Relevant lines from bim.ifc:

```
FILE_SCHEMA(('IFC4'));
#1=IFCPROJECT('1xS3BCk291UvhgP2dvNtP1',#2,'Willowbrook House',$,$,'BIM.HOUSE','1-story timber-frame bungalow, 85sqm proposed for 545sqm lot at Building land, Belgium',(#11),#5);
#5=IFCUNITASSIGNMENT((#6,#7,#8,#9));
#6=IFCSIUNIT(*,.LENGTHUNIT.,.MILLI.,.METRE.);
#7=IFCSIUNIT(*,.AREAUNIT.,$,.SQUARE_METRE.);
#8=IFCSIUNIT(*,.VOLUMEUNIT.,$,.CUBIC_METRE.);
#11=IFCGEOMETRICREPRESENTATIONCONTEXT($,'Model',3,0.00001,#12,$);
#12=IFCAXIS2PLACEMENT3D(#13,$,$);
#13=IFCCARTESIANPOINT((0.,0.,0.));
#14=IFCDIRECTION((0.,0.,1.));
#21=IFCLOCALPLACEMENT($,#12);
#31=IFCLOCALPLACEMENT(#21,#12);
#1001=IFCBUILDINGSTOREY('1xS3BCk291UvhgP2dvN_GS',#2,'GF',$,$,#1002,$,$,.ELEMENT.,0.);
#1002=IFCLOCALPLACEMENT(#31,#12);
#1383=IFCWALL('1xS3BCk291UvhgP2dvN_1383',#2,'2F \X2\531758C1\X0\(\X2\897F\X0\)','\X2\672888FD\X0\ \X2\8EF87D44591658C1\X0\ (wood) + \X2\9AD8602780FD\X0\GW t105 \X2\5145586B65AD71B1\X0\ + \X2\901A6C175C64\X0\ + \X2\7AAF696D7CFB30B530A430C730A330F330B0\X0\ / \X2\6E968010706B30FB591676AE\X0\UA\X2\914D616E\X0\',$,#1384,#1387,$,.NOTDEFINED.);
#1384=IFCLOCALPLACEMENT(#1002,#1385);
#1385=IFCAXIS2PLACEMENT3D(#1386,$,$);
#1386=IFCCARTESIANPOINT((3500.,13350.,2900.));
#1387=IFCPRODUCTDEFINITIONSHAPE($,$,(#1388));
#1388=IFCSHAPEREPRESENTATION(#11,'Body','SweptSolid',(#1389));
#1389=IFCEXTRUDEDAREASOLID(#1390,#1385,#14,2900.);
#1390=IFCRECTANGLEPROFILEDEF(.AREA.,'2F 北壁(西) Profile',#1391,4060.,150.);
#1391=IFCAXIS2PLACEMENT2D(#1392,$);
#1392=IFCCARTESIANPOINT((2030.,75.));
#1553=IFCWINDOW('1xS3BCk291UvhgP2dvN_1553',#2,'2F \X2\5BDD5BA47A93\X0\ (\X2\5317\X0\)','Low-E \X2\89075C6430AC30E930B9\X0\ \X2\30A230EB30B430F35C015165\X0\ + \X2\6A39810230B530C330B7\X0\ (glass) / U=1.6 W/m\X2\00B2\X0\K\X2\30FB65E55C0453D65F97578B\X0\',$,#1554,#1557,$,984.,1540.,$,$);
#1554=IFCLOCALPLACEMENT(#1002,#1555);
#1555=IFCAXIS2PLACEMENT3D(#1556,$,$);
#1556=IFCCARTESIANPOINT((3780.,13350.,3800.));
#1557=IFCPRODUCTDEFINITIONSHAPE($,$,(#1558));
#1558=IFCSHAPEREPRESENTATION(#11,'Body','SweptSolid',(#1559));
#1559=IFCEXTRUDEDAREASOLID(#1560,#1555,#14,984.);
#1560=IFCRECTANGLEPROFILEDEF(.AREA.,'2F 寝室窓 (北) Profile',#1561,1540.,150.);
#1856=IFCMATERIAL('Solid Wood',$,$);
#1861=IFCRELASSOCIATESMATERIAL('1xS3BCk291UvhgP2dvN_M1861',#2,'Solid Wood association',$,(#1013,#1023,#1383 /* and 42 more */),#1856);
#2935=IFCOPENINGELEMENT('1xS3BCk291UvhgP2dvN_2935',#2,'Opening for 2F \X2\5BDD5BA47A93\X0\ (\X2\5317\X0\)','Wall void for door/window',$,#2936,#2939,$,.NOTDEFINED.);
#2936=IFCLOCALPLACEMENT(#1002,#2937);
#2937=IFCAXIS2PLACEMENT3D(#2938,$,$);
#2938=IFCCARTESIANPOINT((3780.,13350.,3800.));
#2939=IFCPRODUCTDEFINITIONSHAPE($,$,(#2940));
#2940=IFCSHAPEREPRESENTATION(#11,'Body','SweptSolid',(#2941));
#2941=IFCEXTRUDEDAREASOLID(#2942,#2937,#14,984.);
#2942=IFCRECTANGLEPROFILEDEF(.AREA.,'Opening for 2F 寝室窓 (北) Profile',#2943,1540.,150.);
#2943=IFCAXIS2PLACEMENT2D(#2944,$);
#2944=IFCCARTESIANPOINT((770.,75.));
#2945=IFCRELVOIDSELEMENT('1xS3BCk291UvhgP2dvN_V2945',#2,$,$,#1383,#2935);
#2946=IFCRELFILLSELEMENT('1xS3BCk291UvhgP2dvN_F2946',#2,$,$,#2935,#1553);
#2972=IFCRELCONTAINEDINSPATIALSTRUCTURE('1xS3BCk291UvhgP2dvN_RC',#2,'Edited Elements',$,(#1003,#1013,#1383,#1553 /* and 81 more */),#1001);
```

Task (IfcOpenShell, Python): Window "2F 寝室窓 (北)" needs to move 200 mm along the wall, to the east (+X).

```python
import ifcopenshell
import ifcopenshell.api.geometry
import ifcopenshell.util.placement

model = ifcopenshell.open("bim.ifc")

window = model.by_guid("1xS3BCk291UvhgP2dvN_1553")
opening = window.FillsVoids[0].RelatingOpeningElement
wall = opening.VoidsElements[0].RelatingBuildingElement

wall_matrix = ifcopenshell.util.placement.get_local_placement(wall.ObjectPlacement)
shift = wall_matrix[:3, 0] * 200.0
before = ifcopenshell.util.placement.get_local_placement(window.ObjectPlacement)[:3, 3].copy()

# The window is not placed relative to its opening, so move both.
for product in (opening, window):
    matrix = ifcopenshell.util.placement.get_local_placement(product.ObjectPlacement)
    matrix[:3, 3] += shift
    ifcopenshell.api.geometry.edit_object_placement(model, product=product, matrix=matrix, is_si=False)

after = ifcopenshell.util.placement.get_local_placement(window.ObjectPlacement)[:3, 3]
print("window moved by", (after - before).round(3) + 0.0)

model.write("bim_updated.ifc")
```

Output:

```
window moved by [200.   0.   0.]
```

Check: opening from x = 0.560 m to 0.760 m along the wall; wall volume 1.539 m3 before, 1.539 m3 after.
